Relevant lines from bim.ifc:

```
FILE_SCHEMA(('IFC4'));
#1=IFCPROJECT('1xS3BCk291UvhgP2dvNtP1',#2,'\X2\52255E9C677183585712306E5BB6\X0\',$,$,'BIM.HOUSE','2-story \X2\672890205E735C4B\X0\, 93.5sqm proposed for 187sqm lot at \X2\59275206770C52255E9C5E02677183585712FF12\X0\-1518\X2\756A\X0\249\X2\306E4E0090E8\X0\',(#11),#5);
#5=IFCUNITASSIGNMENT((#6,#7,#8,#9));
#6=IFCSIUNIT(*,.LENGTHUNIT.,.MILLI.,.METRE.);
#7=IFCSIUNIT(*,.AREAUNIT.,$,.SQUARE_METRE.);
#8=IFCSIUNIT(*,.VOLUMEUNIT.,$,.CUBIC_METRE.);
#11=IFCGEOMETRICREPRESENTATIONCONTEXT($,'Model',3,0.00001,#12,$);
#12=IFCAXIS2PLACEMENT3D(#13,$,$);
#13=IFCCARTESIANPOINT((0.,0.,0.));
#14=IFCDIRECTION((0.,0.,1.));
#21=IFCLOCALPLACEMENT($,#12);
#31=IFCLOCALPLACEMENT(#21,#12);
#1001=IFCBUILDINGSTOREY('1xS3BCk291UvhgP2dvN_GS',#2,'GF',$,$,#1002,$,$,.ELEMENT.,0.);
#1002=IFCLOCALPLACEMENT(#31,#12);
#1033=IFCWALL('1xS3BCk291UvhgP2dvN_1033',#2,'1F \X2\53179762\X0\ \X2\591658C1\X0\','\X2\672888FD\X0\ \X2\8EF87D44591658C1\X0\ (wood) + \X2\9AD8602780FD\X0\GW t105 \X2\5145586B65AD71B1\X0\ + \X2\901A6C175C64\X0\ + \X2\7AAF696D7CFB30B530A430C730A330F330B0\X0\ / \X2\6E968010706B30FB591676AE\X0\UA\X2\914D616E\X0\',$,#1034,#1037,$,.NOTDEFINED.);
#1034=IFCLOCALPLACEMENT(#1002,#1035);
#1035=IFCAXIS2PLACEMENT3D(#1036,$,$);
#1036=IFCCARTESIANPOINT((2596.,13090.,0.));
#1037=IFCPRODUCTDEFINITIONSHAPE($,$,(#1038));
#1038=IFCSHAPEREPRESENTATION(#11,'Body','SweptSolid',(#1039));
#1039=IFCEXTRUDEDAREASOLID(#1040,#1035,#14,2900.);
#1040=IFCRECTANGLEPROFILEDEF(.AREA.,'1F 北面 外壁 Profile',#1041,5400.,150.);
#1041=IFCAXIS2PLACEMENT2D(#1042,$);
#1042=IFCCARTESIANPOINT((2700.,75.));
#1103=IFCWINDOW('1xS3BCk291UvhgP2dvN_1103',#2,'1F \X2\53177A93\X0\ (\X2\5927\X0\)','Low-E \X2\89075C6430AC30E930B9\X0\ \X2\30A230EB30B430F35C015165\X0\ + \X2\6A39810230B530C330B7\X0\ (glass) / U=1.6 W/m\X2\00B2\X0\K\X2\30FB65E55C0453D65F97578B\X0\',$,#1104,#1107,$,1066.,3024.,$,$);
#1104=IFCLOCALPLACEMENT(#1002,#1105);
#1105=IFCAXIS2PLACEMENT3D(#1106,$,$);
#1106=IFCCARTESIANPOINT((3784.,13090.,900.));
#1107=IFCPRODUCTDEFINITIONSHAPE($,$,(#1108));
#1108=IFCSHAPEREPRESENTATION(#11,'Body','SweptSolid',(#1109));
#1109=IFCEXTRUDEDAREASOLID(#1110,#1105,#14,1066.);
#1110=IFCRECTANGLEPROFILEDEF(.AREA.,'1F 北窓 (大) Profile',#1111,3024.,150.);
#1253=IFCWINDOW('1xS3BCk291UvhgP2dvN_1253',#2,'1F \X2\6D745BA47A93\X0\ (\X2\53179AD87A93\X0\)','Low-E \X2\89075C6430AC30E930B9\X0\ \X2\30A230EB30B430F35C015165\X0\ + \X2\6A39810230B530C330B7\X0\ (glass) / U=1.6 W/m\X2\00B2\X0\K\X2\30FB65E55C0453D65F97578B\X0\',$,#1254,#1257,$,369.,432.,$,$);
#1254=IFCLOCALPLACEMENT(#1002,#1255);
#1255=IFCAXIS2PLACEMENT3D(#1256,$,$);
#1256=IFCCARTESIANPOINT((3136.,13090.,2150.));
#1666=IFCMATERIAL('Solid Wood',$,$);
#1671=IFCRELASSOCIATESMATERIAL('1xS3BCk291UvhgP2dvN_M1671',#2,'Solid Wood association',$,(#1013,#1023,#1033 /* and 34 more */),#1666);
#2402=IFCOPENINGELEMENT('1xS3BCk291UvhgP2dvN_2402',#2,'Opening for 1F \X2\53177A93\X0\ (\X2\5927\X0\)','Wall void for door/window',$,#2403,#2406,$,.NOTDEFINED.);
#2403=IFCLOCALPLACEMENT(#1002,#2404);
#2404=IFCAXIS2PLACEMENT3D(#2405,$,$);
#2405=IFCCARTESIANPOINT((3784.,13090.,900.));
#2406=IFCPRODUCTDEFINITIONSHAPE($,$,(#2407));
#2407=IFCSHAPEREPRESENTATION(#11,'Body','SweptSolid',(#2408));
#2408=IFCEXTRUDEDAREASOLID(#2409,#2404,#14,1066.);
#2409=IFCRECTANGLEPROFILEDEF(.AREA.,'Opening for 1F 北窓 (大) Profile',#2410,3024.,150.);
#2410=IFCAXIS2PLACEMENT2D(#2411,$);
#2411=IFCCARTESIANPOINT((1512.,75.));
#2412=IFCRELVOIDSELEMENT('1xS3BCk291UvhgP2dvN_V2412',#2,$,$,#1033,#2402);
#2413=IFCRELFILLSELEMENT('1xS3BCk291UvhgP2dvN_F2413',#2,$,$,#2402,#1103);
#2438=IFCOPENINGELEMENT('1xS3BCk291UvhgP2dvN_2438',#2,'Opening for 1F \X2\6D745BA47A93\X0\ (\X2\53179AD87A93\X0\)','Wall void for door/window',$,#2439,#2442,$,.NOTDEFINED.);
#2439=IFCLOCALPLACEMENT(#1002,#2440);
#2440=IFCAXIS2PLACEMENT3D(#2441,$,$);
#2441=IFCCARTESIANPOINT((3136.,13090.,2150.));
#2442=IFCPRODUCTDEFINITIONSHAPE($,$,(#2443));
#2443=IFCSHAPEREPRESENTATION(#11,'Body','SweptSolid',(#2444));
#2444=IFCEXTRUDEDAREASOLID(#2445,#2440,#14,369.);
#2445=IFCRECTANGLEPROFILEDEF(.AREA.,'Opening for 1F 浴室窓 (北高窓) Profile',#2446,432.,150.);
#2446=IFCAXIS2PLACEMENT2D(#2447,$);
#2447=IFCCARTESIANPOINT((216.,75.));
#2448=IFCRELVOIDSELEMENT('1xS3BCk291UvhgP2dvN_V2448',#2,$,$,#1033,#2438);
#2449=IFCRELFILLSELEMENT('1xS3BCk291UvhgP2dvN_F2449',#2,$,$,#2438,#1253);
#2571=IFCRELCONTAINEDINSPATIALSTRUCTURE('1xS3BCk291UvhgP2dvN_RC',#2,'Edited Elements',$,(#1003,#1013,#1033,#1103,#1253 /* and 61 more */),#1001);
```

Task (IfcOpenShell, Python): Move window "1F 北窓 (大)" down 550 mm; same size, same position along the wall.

```python
import numpy as np
import ifcopenshell
import ifcopenshell.api.geometry
import ifcopenshell.util.placement
import ifcopenshell.util.unit

model = ifcopenshell.open("bim.ifc")
unit_scale = ifcopenshell.util.unit.calculate_unit_scale(model)

window = model.by_id(1103)
opening = window.FillsVoids[0].RelatingOpeningElement
dz = -0.55 / unit_scale

shift = np.array([0.0, 0.0, dz])
# The window is not placed relative to its opening, so move both.
for product in (opening, window):
    matrix = ifcopenshell.util.placement.get_local_placement(product.ObjectPlacement)
    matrix[:3, 3] += shift
    ifcopenshell.api.geometry.edit_object_placement(model, product=product, matrix=matrix, is_si=False)

print(f"moved by {dz * unit_scale:+.3f} m")

model.write("bim_v2.ifc")
```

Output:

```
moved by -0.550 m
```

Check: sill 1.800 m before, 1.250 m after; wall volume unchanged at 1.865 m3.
